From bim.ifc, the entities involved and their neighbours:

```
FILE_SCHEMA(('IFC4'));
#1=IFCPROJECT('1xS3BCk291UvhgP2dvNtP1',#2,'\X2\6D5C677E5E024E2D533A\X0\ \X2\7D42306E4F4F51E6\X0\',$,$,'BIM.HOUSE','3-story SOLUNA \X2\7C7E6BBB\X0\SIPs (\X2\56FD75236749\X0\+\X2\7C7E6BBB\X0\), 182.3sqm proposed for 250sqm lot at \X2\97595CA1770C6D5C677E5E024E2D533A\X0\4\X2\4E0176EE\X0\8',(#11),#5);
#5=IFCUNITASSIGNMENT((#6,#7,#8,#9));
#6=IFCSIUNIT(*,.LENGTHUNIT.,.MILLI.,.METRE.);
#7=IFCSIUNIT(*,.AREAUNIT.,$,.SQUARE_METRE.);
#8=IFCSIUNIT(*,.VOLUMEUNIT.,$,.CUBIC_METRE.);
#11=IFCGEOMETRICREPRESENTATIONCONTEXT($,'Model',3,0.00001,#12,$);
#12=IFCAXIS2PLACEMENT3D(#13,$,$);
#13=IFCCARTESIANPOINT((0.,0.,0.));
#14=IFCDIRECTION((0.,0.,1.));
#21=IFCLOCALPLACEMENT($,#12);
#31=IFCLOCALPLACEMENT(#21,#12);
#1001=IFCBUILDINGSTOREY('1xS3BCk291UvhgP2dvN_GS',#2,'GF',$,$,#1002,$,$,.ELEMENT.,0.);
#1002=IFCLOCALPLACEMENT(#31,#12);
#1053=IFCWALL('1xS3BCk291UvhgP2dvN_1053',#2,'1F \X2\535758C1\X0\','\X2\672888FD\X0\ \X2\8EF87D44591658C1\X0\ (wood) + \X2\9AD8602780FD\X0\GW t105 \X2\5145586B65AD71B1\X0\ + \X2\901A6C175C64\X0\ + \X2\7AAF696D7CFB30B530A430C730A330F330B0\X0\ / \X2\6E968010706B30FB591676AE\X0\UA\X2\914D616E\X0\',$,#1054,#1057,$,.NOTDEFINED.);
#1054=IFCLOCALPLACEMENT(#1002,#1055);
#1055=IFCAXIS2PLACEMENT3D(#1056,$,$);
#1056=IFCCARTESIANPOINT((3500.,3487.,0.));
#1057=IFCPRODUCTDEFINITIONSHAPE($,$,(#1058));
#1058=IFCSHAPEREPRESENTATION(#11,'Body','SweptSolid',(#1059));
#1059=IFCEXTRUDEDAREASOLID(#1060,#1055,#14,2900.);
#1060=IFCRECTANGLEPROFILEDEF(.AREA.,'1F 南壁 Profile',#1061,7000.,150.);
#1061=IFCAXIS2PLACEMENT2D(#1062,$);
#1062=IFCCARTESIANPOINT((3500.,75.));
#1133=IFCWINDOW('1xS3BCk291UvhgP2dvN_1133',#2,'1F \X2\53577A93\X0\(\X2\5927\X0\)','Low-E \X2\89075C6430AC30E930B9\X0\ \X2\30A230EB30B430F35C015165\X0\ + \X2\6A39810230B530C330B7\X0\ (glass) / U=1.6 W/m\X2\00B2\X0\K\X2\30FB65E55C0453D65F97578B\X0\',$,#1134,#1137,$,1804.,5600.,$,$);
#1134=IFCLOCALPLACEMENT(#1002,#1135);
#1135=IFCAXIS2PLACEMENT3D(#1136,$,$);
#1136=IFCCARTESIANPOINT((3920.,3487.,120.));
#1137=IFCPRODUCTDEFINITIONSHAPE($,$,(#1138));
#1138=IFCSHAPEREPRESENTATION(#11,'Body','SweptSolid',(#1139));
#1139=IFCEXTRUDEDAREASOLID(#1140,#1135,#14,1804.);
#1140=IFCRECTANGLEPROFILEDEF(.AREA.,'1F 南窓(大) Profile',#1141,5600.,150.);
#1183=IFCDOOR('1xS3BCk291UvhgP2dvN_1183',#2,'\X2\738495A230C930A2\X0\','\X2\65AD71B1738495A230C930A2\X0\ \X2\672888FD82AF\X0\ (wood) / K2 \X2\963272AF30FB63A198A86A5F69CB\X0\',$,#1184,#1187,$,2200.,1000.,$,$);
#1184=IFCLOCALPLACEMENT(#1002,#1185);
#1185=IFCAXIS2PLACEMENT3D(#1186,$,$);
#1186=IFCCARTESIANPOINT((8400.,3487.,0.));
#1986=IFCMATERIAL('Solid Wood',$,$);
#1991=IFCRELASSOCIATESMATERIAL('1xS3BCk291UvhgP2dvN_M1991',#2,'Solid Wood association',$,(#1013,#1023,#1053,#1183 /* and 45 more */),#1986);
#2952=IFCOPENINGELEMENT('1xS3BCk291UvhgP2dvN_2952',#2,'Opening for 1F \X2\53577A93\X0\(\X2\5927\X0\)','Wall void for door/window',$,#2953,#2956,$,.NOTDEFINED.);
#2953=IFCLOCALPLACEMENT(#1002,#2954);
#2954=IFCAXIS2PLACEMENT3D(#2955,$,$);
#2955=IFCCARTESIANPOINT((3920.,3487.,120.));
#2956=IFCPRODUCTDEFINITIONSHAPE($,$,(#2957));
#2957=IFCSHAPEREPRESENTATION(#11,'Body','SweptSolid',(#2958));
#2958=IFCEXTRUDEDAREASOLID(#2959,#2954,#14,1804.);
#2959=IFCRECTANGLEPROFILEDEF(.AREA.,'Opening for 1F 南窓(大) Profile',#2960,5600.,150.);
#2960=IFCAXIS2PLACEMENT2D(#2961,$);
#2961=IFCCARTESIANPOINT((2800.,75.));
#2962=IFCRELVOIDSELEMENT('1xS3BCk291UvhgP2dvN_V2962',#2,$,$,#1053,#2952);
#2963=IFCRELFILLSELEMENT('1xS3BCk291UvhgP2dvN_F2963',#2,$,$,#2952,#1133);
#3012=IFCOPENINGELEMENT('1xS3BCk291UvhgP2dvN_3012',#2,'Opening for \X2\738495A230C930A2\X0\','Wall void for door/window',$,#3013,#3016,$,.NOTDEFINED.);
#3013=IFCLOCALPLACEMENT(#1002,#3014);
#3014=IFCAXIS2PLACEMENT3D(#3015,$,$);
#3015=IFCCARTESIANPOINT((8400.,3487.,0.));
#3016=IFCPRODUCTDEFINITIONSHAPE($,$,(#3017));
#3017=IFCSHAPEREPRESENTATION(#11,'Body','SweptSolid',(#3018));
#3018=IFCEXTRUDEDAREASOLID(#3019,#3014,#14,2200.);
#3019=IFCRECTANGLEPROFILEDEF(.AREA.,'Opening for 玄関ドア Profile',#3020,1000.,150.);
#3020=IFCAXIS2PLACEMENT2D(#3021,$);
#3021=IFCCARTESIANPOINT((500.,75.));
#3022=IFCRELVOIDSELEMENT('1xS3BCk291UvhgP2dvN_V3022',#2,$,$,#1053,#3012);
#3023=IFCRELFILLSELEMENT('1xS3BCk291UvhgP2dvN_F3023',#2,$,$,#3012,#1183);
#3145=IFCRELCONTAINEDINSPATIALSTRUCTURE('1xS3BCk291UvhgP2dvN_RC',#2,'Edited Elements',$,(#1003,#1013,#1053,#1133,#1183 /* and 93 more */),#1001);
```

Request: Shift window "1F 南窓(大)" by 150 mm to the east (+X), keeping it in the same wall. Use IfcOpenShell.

```python
import ifcopenshell
import ifcopenshell.api.geometry
import ifcopenshell.util.placement
import ifcopenshell.util.unit

model = ifcopenshell.open("bim.ifc")
unit_scale = ifcopenshell.util.unit.calculate_unit_scale(model)

window = model.by_id(1133)
opening = window.FillsVoids[0].RelatingOpeningElement
wall = opening.VoidsElements[0].RelatingBuildingElement

wall_matrix = ifcopenshell.util.placement.get_local_placement(wall.ObjectPlacement)
shift = wall_matrix[:3, 0] * 0.15 / unit_scale
before = ifcopenshell.util.placement.get_local_placement(window.ObjectPlacement)[:3, 3].copy()

# The window is not placed relative to its opening, so move both.
for product in (opening, window):
    matrix = ifcopenshell.util.placement.get_local_placement(product.ObjectPlacement)
    matrix[:3, 3] += shift
    ifcopenshell.api.geometry.edit_object_placement(model, product=product, matrix=matrix, is_si=False)

after = ifcopenshell.util.placement.get_local_placement(window.ObjectPlacement)[:3, 3]
print("window moved by", (after - before).round(3) + 0.0)

model.write("bim_rev.ifc")
```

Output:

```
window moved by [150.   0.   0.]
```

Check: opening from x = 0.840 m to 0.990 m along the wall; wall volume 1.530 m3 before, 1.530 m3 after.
